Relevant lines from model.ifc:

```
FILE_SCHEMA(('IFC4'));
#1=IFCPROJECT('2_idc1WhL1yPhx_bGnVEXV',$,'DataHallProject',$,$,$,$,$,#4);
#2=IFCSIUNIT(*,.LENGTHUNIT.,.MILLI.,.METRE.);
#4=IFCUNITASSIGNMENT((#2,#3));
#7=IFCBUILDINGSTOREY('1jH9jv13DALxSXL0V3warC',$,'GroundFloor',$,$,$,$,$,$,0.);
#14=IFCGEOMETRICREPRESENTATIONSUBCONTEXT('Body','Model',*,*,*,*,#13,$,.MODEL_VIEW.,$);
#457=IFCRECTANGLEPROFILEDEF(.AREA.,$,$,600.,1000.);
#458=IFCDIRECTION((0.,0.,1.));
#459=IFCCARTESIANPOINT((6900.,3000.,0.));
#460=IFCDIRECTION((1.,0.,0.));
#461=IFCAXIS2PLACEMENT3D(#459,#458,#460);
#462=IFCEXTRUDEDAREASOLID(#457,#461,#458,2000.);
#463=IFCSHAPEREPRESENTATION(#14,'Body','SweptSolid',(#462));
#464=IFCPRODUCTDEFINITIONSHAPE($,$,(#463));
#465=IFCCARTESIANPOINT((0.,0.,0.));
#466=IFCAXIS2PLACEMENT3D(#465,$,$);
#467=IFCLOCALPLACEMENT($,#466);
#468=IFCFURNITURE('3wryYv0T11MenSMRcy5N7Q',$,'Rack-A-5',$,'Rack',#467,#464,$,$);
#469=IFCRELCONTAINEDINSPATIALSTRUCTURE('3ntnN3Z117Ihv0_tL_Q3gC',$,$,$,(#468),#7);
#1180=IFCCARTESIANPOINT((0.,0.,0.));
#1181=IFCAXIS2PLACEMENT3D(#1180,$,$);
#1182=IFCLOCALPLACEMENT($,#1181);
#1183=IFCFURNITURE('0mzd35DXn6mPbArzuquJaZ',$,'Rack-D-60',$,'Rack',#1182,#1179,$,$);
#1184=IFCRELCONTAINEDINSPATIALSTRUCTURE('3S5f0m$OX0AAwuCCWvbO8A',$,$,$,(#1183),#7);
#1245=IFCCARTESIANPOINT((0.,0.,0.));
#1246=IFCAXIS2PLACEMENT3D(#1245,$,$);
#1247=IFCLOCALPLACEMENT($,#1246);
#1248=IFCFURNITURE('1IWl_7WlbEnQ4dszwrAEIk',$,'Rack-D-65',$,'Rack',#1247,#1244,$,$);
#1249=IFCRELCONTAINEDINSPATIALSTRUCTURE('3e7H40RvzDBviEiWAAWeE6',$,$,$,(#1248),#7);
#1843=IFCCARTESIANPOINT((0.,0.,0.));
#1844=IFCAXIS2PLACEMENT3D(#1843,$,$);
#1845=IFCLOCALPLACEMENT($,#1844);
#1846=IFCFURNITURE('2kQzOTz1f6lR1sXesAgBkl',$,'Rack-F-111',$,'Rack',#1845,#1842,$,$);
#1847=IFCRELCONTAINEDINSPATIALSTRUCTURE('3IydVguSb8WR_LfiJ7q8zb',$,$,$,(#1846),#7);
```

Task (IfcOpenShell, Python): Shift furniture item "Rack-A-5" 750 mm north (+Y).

```python
import ifcopenshell
import ifcopenshell.api.geometry
import ifcopenshell.util.placement
import ifcopenshell.util.unit

model = ifcopenshell.open("model.ifc")
unit_scale = ifcopenshell.util.unit.calculate_unit_scale(model)

item = model.by_id(468)
matrix = ifcopenshell.util.placement.get_local_placement(item.ObjectPlacement)
matrix[1, 3] += 0.75 / unit_scale
ifcopenshell.api.geometry.edit_object_placement(model, product=item, matrix=matrix, is_si=False)

print(ifcopenshell.util.placement.get_local_placement(item.ObjectPlacement).round(3) + 0.0)

model.write("model_rev.ifc")
```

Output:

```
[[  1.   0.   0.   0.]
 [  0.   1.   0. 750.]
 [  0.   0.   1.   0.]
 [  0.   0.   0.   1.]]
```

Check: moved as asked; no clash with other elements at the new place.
